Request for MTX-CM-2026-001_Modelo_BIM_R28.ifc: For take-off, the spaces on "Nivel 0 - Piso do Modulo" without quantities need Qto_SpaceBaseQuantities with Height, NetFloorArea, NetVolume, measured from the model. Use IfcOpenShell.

First a look at what the model holds.

```python
import ifcopenshell
import ifcopenshell.util.element
import ifcopenshell.util.unit

model = ifcopenshell.open("MTX-CM-2026-001_Modelo_BIM_R28.ifc")
print(model.schema)
for unit_type in ("LENGTHUNIT", "AREAUNIT", "VOLUMEUNIT"):
    print(unit_type, ifcopenshell.util.unit.calculate_unit_scale(model, unit_type))
storey = next(s for s in model.by_type("IfcBuildingStorey") if s.Name == "Nivel 0 - Piso do Modulo")
spaces = [e for e in ifcopenshell.util.element.get_decomposition(storey) if e.is_a("IfcSpace")]
for e in sorted(spaces, key=lambda e: e.id()):
    print(e.id(), e.is_a(), e.Name, list(ifcopenshell.util.element.get_psets(e, qtos_only=True)), sep=" | ")
```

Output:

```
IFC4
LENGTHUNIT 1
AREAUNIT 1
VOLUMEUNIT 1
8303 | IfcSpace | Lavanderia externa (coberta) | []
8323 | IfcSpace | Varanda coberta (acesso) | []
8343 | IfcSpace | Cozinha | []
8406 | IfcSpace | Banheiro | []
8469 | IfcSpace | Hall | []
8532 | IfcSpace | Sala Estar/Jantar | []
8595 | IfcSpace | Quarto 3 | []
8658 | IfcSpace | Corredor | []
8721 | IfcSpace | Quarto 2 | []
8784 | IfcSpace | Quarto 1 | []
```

```python
import ifcopenshell
import ifcopenshell.api.pset
import ifcopenshell.geom
import ifcopenshell.util.element
import ifcopenshell.util.shape
import ifcopenshell.util.unit

model = ifcopenshell.open("MTX-CM-2026-001_Modelo_BIM_R28.ifc")
unit_scale = ifcopenshell.util.unit.calculate_unit_scale(model)
area_scale = ifcopenshell.util.unit.calculate_unit_scale(model, "AREAUNIT")
volume_scale = ifcopenshell.util.unit.calculate_unit_scale(model, "VOLUMEUNIT")
settings = ifcopenshell.geom.settings()

storey = next(s for s in model.by_type("IfcBuildingStorey") if s.Name == "Nivel 0 - Piso do Modulo")
spaces = [e for e in ifcopenshell.util.element.get_decomposition(storey) if e.is_a("IfcSpace")]

for e in sorted(spaces, key=lambda e: e.id()):
    if ifcopenshell.util.element.get_psets(e, qtos_only=True, should_inherit=False):
        continue
    # Geometry comes back in metres, in the element's own axes.
    shape = ifcopenshell.geom.create_shape(settings, e)
    values = {
        "Height": ifcopenshell.util.shape.get_z(shape.geometry) / unit_scale,
        "NetFloorArea": ifcopenshell.util.shape.get_footprint_area(shape.geometry) / area_scale,
        "NetVolume": ifcopenshell.util.shape.get_volume(shape.geometry) / volume_scale,
    }
    qto = ifcopenshell.api.pset.add_qto(model, product=e, name="Qto_SpaceBaseQuantities")
    ifcopenshell.api.pset.edit_qto(model, qto=qto, properties=values)
    print(e.id(), {k: round(v, 3) for k, v in values.items()})

model.write("MTX-CM-2026-001_Modelo_BIM_R28_rev.ifc")
```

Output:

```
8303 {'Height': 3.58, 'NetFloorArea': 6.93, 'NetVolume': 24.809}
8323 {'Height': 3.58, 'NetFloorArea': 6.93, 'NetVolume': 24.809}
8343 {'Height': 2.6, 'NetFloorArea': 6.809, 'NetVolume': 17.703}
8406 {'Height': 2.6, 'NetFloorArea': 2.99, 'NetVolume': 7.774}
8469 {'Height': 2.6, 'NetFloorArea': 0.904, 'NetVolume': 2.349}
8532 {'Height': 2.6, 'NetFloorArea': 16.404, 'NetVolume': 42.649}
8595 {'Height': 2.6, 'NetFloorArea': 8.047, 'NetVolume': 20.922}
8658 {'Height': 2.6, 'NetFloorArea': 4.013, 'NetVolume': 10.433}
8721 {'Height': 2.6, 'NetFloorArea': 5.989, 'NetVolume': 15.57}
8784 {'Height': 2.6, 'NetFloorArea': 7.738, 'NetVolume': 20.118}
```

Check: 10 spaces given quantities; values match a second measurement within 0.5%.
